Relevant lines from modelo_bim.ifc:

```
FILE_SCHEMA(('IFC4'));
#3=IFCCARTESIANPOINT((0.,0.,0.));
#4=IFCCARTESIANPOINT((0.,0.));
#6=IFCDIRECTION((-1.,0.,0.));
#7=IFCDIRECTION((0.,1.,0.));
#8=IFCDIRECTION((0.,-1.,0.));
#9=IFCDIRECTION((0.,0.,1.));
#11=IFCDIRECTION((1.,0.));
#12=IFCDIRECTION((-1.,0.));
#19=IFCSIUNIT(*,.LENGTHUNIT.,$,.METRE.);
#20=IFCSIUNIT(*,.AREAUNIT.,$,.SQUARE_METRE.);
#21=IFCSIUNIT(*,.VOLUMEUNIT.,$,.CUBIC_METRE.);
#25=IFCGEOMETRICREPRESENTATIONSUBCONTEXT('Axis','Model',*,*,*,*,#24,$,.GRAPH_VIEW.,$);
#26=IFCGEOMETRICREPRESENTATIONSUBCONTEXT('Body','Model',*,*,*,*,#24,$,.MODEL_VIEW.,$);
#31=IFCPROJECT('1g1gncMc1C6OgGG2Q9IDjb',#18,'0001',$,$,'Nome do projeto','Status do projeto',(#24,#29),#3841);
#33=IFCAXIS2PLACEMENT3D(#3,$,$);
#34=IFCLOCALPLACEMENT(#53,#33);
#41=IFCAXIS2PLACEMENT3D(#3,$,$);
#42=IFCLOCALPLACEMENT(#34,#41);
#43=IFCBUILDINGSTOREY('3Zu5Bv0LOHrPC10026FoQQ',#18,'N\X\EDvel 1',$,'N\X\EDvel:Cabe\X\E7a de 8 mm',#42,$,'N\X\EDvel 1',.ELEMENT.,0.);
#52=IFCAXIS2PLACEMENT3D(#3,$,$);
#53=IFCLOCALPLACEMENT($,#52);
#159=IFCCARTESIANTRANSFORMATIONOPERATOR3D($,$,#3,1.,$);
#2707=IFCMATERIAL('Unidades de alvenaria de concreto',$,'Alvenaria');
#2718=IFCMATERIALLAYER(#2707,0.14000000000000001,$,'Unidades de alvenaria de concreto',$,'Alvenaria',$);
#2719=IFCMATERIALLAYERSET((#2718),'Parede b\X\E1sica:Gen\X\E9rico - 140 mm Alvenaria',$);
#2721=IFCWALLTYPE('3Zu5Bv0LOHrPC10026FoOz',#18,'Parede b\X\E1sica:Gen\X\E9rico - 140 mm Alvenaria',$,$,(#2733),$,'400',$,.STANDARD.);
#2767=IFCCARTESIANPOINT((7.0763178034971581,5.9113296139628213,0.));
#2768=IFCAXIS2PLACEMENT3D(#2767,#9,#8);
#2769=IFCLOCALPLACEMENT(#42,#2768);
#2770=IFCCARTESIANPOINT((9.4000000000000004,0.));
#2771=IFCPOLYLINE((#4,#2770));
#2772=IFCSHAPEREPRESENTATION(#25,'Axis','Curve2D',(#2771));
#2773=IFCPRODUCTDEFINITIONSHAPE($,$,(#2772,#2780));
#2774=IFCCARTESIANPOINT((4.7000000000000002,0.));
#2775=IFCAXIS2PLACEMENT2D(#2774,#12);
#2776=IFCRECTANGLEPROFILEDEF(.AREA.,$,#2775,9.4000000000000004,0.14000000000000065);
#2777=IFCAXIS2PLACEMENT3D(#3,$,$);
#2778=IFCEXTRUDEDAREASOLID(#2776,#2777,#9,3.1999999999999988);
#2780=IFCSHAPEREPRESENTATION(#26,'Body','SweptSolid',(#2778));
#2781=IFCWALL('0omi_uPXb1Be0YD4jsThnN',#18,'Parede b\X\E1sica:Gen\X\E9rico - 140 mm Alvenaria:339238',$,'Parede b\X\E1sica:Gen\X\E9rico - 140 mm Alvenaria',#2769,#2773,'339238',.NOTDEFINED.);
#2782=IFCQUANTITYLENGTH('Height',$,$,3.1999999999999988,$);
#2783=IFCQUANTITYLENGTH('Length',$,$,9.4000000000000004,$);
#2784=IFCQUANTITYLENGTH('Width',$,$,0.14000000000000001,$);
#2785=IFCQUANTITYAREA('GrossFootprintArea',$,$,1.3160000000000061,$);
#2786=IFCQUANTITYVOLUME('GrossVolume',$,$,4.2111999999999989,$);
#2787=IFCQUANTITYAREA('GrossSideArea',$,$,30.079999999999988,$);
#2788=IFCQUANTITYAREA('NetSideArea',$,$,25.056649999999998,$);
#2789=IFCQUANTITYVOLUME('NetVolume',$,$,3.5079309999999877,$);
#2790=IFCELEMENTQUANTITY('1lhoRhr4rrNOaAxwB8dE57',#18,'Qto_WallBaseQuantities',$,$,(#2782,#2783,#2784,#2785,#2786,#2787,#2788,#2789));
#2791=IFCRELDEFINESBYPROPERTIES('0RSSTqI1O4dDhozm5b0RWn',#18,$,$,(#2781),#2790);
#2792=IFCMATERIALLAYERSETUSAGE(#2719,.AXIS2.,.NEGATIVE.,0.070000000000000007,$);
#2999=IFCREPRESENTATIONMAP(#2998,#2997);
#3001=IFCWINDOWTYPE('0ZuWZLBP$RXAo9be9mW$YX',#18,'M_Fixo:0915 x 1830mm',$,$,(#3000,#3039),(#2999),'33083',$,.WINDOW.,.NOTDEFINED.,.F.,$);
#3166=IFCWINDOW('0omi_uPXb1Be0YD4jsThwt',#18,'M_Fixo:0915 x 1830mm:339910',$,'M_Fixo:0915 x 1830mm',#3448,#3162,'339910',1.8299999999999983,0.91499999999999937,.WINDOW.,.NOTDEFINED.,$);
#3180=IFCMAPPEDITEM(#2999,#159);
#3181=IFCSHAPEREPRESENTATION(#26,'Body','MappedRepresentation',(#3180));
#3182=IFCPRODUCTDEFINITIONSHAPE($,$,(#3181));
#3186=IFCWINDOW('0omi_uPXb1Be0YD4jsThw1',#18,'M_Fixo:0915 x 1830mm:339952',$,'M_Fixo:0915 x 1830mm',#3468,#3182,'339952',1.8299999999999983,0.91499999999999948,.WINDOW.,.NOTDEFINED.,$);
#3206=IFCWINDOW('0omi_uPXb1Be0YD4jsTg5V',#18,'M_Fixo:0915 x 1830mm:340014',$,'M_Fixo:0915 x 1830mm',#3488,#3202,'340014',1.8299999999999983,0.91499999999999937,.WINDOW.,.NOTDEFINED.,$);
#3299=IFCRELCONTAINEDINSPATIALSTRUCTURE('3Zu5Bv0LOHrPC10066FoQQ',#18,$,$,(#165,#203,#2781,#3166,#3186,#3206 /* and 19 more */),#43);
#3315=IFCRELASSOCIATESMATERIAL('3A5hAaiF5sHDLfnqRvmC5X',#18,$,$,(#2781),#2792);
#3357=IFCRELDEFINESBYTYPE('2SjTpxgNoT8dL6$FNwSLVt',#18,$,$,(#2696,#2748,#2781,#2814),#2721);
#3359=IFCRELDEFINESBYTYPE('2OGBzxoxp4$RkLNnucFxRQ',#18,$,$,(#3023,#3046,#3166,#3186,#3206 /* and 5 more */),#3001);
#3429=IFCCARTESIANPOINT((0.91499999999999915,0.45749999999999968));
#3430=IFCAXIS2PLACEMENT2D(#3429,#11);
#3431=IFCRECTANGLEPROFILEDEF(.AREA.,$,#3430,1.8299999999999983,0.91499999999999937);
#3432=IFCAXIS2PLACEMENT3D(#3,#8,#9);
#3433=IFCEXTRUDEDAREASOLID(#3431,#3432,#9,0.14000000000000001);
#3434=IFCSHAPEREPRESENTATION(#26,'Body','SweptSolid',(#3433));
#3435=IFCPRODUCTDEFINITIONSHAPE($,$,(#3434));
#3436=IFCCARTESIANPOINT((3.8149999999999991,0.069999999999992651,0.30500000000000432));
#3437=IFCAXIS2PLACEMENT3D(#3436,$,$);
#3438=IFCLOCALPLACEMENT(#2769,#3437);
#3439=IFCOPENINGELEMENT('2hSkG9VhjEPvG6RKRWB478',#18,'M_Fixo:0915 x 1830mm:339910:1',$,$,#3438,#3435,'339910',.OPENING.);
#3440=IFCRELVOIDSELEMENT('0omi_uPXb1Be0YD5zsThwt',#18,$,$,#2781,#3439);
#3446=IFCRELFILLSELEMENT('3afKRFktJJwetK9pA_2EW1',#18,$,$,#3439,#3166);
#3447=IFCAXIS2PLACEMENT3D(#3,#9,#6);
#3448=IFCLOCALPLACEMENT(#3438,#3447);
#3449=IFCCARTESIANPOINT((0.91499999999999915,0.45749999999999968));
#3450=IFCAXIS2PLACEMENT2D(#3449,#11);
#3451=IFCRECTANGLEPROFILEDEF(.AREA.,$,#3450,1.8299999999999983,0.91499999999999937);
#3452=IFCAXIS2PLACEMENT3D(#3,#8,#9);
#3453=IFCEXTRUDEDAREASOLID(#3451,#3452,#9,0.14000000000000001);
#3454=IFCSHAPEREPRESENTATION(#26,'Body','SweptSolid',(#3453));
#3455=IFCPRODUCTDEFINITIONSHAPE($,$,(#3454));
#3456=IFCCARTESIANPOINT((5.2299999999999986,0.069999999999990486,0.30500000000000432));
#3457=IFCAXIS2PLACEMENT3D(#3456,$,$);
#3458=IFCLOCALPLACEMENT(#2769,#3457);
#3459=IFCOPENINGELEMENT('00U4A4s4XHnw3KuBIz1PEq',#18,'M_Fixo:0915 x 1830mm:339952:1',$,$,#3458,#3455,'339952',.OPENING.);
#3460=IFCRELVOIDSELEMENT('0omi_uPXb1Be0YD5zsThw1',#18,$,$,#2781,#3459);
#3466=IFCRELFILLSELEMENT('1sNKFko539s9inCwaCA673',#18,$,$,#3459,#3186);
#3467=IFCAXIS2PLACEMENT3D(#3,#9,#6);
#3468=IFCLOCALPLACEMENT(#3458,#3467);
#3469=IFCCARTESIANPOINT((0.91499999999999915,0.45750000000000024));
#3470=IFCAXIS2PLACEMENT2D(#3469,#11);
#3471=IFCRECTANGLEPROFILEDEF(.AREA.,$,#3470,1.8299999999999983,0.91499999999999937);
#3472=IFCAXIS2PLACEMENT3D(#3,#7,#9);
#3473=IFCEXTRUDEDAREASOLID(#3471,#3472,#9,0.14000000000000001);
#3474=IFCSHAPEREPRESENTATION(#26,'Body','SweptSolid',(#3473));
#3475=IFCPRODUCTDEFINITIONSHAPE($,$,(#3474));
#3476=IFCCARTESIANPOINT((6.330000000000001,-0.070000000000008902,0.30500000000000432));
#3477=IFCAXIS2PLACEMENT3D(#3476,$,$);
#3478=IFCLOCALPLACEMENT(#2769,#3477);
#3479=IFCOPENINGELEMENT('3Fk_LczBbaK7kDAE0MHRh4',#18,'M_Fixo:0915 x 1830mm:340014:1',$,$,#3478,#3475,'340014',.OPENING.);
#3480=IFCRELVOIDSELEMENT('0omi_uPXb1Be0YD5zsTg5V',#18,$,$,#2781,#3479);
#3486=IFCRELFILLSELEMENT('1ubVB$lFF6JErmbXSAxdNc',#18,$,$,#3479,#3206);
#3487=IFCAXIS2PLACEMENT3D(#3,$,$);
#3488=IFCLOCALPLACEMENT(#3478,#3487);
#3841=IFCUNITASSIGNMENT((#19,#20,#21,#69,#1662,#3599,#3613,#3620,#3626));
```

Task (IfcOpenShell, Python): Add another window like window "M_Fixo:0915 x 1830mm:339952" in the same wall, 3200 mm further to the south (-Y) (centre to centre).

```python
import ifcopenshell
import ifcopenshell.api.feature
import ifcopenshell.api.geometry
import ifcopenshell.api.pset
import ifcopenshell.api.root
import ifcopenshell.geom
import ifcopenshell.util.element
import ifcopenshell.util.placement
import ifcopenshell.util.shape
import ifcopenshell.util.unit

model = ifcopenshell.open("modelo_bim.ifc")
unit_scale = ifcopenshell.util.unit.calculate_unit_scale(model)
area_scale = ifcopenshell.util.unit.calculate_unit_scale(model, "AREAUNIT")
volume_scale = ifcopenshell.util.unit.calculate_unit_scale(model, "VOLUMEUNIT")
settings = ifcopenshell.geom.settings()


def volume(element):
    """Net volume in cubic metres, openings subtracted."""
    shape = ifcopenshell.geom.create_shape(settings, element)
    return ifcopenshell.util.shape.get_volume(shape.geometry)


def reuse_history(source, copy):
    """copy_class also copies each property set's owner history, people and application; keep the originals."""
    for rel in copy.IsDefinedBy:
        if rel.is_a("IfcRelDefinesByProperties") and (history := rel.RelatingPropertyDefinition.OwnerHistory):
            rel.RelatingPropertyDefinition.OwnerHistory = source.OwnerHistory
            ifcopenshell.util.element.remove_deep2(model, history)


window = model.by_guid("0omi_uPXb1Be0YD4jsThw1")
opening = window.FillsVoids[0].RelatingOpeningElement
wall = opening.VoidsElements[0].RelatingBuildingElement
before = volume(wall)
shift = ifcopenshell.util.placement.get_local_placement(wall.ObjectPlacement)[:3, 0] * 3.2 / unit_scale

# copy_class copies the void relationship, type, container and properties, but no geometry.
new_opening = ifcopenshell.api.root.copy_class(model, product=opening)
new_opening.Representation = ifcopenshell.util.element.copy_deep(
    model, opening.Representation, exclude=["IfcGeometricRepresentationContext", "IfcRepresentationMap"]
)
new_opening.Name = "M_Fixo:0915 x 1830mm"
new_opening.Tag = None
reuse_history(opening, new_opening)
new_window = ifcopenshell.api.root.copy_class(model, product=window)
new_window.Representation = ifcopenshell.util.element.copy_deep(
    model, window.Representation, exclude=["IfcGeometricRepresentationContext", "IfcRepresentationMap"]
)
new_window.Name = "M_Fixo:0915 x 1830mm"
new_window.Tag = None
reuse_history(window, new_window)
ifcopenshell.api.feature.add_filling(model, opening=new_opening, element=new_window)

for old, new in ((opening, new_opening), (window, new_window)):
    matrix = ifcopenshell.util.placement.get_local_placement(old.ObjectPlacement)
    matrix[:3, 3] += shift
    ifcopenshell.api.geometry.edit_object_placement(model, product=new, matrix=matrix, is_si=False)

after = volume(wall)
thickness = 0.14  # wall thickness in metres

# Update the wall's stored quantities.
qto = model.by_id(ifcopenshell.util.element.get_pset(wall, "Qto_WallBaseQuantities", should_inherit=False)["id"])
ifcopenshell.api.pset.edit_qto(model, qto=qto, properties={
    "NetSideArea": after / thickness / area_scale,
    "NetVolume": after / volume_scale,
})

print(f"wall volume {before:.3f} -> {after:.3f} m3")

model.write("modelo_bim_updated.ifc")
```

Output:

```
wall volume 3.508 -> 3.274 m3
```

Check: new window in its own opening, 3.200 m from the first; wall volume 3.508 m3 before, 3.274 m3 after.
